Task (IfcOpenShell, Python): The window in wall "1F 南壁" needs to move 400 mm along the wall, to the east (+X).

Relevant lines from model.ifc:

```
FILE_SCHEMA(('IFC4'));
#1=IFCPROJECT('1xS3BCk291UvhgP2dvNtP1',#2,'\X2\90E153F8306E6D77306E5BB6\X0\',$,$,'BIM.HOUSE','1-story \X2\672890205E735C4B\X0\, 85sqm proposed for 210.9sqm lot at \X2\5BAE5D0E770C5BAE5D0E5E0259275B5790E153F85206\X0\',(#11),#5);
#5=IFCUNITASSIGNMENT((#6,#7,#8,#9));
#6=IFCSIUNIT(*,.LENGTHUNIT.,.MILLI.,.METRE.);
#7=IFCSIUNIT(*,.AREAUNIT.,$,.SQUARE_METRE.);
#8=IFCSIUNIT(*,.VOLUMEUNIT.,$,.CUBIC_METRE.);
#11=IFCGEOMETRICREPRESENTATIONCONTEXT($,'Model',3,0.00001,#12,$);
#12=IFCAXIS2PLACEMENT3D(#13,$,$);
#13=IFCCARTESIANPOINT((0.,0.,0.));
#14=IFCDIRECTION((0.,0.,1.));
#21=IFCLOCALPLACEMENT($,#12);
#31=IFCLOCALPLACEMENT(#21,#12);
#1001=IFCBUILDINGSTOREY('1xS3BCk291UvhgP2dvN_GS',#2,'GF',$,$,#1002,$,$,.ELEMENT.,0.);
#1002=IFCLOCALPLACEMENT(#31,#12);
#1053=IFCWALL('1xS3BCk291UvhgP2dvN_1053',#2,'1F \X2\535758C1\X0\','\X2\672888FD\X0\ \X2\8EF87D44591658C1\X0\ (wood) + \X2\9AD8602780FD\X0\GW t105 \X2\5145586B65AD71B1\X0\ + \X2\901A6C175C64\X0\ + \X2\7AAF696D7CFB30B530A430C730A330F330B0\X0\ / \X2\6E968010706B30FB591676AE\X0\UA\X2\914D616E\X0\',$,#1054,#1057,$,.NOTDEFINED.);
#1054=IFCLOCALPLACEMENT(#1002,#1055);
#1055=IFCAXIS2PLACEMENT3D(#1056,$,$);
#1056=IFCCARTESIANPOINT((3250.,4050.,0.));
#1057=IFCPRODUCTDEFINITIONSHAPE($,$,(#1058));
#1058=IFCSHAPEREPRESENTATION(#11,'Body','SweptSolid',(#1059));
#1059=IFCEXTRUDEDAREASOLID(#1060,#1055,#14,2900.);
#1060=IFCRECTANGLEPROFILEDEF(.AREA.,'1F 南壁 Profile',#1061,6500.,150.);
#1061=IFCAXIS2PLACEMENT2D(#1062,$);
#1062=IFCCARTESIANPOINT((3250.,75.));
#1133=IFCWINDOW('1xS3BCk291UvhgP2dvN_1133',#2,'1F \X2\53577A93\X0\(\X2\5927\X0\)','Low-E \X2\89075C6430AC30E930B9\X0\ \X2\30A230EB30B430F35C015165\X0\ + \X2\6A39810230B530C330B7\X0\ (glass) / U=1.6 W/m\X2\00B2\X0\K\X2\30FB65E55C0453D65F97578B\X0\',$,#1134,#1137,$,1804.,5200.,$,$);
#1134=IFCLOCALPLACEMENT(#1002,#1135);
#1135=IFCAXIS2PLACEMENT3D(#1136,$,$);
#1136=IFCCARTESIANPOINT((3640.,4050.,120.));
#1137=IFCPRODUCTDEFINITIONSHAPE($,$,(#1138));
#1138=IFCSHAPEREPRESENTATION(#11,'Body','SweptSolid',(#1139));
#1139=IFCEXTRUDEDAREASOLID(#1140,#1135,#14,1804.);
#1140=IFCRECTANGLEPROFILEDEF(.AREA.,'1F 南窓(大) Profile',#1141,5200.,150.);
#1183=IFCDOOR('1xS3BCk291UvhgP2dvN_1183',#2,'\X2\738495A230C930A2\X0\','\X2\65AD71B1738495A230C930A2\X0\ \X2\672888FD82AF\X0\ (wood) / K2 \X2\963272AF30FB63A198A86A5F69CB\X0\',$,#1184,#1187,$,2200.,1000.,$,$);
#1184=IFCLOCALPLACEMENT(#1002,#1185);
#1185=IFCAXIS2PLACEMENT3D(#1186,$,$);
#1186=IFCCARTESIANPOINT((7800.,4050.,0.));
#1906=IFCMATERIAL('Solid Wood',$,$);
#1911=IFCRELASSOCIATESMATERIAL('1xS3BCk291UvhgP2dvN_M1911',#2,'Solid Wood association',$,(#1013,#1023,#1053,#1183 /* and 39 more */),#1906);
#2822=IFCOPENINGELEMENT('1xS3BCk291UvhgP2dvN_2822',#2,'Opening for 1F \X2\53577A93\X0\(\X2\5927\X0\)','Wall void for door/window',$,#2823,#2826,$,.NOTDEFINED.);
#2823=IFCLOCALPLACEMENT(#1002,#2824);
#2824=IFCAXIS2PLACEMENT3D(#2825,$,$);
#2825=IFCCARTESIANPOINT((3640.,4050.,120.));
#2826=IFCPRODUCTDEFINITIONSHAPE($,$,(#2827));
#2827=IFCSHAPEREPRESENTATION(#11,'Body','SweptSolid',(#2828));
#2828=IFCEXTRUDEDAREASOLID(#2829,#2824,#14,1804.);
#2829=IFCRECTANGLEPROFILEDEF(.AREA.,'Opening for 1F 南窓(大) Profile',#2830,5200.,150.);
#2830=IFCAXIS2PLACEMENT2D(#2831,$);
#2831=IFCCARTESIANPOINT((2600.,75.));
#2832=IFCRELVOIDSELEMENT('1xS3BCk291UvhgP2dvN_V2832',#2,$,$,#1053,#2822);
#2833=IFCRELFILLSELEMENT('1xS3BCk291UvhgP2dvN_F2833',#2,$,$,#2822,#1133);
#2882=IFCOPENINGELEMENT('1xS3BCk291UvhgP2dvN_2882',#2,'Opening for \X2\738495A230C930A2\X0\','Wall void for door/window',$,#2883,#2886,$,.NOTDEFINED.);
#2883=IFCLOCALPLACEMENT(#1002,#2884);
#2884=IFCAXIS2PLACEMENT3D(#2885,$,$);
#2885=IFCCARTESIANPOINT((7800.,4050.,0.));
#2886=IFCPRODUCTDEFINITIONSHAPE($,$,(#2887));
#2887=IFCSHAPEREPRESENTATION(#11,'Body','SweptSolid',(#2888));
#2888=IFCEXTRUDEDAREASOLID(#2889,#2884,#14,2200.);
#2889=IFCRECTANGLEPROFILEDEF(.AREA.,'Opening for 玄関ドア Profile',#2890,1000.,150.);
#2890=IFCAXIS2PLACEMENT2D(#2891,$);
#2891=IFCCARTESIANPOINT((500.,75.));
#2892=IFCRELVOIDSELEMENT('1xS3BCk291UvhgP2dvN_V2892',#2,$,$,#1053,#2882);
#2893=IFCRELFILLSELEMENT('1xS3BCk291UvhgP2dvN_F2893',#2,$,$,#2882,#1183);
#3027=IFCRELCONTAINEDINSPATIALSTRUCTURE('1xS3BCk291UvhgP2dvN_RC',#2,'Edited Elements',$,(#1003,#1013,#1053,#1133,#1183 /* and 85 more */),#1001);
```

```python
import ifcopenshell
import ifcopenshell.api.geometry
import ifcopenshell.util.placement

model = ifcopenshell.open("model.ifc")

window = model.by_id(1133)
opening = window.FillsVoids[0].RelatingOpeningElement
wall = opening.VoidsElements[0].RelatingBuildingElement

wall_matrix = ifcopenshell.util.placement.get_local_placement(wall.ObjectPlacement)
shift = wall_matrix[:3, 0] * 400.0
before = ifcopenshell.util.placement.get_local_placement(window.ObjectPlacement)[:3, 3].copy()

# The window is not placed relative to its opening, so move both.
for product in (opening, window):
    matrix = ifcopenshell.util.placement.get_local_placement(product.ObjectPlacement)
    matrix[:3, 3] += shift
    ifcopenshell.api.geometry.edit_object_placement(model, product=product, matrix=matrix, is_si=False)

after = ifcopenshell.util.placement.get_local_placement(window.ObjectPlacement)[:3, 3]
print("window moved by", (after - before).round(3) + 0.0)

model.write("model_edited.ifc")
```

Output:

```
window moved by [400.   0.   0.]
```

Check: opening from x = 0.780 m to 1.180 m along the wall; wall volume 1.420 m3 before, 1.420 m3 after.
